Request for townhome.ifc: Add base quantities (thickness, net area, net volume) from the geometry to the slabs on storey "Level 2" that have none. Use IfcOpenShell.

First a look at what the model holds.

```python
import ifcopenshell
import ifcopenshell.util.element
import ifcopenshell.util.unit

model = ifcopenshell.open("townhome.ifc")
print(model.schema)
for unit_type in ("LENGTHUNIT", "AREAUNIT", "VOLUMEUNIT"):
    print(unit_type, ifcopenshell.util.unit.calculate_unit_scale(model, unit_type))
storey = next(s for s in model.by_type("IfcBuildingStorey") if s.Name == "Level 2")
slabs = [e for e in ifcopenshell.util.element.get_decomposition(storey) if e.is_a("IfcSlab")]
for e in sorted(slabs, key=lambda e: e.id()):
    print(e.id(), e.is_a(), e.Name, list(ifcopenshell.util.element.get_psets(e, qtos_only=True)), sep=" | ")
```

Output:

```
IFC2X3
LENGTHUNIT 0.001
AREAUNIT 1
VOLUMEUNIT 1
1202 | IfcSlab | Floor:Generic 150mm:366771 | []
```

```python
import ifcopenshell
import ifcopenshell.api.pset
import ifcopenshell.geom
import ifcopenshell.util.element
import ifcopenshell.util.shape
import ifcopenshell.util.unit

model = ifcopenshell.open("townhome.ifc")
unit_scale = ifcopenshell.util.unit.calculate_unit_scale(model)
area_scale = ifcopenshell.util.unit.calculate_unit_scale(model, "AREAUNIT")
volume_scale = ifcopenshell.util.unit.calculate_unit_scale(model, "VOLUMEUNIT")
settings = ifcopenshell.geom.settings()

storey = next(s for s in model.by_type("IfcBuildingStorey") if s.Name == "Level 2")
slabs = [e for e in ifcopenshell.util.element.get_decomposition(storey) if e.is_a("IfcSlab")]

for e in sorted(slabs, key=lambda e: e.id()):
    if ifcopenshell.util.element.get_psets(e, qtos_only=True, should_inherit=False):
        continue
    # Geometry comes back in metres, in the element's own axes.
    shape = ifcopenshell.geom.create_shape(settings, e)
    values = {
        "Width": ifcopenshell.util.shape.get_z(shape.geometry) / unit_scale,
        "NetArea": ifcopenshell.util.shape.get_footprint_area(shape.geometry) / area_scale,
        "NetVolume": ifcopenshell.util.shape.get_volume(shape.geometry) / volume_scale,
    }
    qto = ifcopenshell.api.pset.add_qto(model, product=e, name="BaseQuantities")
    ifcopenshell.api.pset.edit_qto(model, qto=qto, properties=values)
    print(e.id(), {k: round(v, 3) for k, v in values.items()})

model.write("townhome_edited.ifc")
```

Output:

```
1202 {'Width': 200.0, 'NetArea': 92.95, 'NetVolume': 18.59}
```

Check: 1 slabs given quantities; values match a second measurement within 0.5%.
